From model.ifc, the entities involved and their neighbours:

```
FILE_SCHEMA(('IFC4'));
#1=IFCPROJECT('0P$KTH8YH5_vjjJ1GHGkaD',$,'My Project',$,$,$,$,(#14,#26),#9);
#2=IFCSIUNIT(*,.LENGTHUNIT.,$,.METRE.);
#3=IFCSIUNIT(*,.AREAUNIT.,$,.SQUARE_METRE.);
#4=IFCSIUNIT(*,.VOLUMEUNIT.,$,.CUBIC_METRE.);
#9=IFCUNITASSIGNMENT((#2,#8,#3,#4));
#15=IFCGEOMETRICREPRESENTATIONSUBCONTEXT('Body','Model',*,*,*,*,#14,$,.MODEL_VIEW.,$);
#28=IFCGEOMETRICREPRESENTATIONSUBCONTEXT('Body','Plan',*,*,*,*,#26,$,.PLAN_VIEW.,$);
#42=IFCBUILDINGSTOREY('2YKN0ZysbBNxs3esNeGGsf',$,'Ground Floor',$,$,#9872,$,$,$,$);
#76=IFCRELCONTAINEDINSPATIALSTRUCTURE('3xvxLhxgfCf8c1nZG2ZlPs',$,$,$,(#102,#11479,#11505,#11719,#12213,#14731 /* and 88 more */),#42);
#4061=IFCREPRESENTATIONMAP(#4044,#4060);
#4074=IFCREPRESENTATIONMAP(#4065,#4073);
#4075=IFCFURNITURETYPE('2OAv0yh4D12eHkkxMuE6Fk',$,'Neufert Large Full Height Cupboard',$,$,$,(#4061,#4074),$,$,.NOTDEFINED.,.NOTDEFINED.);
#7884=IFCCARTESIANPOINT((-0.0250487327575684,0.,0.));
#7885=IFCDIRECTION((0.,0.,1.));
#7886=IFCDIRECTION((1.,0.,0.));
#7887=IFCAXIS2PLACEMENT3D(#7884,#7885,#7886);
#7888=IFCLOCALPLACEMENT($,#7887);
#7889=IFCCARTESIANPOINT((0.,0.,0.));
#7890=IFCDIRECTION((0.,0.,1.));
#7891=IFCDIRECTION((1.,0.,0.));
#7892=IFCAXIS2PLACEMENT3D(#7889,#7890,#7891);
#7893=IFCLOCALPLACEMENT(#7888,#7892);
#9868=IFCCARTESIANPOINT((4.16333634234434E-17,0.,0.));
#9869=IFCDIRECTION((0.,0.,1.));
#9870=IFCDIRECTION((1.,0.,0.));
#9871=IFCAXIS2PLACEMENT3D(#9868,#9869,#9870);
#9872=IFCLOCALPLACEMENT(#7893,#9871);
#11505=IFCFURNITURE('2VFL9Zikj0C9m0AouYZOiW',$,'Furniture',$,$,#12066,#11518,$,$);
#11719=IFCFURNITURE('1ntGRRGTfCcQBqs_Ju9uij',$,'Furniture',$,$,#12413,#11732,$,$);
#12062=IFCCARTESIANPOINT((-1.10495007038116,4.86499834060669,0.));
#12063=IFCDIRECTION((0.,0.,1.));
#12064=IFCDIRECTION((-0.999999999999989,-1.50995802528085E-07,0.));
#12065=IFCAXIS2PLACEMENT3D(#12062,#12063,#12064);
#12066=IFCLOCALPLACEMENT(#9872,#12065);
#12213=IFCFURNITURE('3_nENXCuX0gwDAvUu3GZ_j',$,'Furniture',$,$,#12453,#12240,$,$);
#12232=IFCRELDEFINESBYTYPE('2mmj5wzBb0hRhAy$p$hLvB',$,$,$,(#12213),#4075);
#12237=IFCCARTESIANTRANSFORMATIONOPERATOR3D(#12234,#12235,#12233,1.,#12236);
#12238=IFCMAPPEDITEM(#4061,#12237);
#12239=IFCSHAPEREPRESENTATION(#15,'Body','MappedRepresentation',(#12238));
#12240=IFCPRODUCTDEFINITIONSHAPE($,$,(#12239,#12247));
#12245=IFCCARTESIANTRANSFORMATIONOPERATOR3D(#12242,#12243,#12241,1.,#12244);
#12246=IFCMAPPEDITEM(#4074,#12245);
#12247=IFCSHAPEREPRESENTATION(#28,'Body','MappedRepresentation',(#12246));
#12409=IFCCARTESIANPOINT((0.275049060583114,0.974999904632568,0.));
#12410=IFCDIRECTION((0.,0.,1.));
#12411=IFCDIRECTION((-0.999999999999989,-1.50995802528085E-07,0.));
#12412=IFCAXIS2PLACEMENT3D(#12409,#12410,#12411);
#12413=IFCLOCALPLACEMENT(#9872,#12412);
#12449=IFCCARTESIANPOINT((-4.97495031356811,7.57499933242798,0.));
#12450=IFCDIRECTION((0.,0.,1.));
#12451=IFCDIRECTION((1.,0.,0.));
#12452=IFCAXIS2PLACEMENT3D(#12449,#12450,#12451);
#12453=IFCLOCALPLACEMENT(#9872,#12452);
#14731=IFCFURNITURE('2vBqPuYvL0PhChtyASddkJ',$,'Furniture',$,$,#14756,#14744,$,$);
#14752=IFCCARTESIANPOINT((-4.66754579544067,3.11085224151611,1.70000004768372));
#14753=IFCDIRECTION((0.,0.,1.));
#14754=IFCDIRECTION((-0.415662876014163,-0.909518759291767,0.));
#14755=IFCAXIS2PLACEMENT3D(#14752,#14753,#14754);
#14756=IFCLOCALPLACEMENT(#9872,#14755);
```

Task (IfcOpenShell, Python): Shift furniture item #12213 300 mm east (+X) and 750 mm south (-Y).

```python
import ifcopenshell
import ifcopenshell.api.geometry
import ifcopenshell.util.placement

model = ifcopenshell.open("model.ifc")

item = model.by_id(12213)
matrix = ifcopenshell.util.placement.get_local_placement(item.ObjectPlacement)
matrix[0, 3] += 0.3
matrix[1, 3] -= 0.75
ifcopenshell.api.geometry.edit_object_placement(model, product=item, matrix=matrix, is_si=False)

print(ifcopenshell.util.placement.get_local_placement(item.ObjectPlacement).round(3) + 0.0)

model.write("model_rev.ifc")
```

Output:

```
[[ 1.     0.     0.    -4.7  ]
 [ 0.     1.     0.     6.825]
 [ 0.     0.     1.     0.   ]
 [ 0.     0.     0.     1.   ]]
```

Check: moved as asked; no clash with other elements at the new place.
